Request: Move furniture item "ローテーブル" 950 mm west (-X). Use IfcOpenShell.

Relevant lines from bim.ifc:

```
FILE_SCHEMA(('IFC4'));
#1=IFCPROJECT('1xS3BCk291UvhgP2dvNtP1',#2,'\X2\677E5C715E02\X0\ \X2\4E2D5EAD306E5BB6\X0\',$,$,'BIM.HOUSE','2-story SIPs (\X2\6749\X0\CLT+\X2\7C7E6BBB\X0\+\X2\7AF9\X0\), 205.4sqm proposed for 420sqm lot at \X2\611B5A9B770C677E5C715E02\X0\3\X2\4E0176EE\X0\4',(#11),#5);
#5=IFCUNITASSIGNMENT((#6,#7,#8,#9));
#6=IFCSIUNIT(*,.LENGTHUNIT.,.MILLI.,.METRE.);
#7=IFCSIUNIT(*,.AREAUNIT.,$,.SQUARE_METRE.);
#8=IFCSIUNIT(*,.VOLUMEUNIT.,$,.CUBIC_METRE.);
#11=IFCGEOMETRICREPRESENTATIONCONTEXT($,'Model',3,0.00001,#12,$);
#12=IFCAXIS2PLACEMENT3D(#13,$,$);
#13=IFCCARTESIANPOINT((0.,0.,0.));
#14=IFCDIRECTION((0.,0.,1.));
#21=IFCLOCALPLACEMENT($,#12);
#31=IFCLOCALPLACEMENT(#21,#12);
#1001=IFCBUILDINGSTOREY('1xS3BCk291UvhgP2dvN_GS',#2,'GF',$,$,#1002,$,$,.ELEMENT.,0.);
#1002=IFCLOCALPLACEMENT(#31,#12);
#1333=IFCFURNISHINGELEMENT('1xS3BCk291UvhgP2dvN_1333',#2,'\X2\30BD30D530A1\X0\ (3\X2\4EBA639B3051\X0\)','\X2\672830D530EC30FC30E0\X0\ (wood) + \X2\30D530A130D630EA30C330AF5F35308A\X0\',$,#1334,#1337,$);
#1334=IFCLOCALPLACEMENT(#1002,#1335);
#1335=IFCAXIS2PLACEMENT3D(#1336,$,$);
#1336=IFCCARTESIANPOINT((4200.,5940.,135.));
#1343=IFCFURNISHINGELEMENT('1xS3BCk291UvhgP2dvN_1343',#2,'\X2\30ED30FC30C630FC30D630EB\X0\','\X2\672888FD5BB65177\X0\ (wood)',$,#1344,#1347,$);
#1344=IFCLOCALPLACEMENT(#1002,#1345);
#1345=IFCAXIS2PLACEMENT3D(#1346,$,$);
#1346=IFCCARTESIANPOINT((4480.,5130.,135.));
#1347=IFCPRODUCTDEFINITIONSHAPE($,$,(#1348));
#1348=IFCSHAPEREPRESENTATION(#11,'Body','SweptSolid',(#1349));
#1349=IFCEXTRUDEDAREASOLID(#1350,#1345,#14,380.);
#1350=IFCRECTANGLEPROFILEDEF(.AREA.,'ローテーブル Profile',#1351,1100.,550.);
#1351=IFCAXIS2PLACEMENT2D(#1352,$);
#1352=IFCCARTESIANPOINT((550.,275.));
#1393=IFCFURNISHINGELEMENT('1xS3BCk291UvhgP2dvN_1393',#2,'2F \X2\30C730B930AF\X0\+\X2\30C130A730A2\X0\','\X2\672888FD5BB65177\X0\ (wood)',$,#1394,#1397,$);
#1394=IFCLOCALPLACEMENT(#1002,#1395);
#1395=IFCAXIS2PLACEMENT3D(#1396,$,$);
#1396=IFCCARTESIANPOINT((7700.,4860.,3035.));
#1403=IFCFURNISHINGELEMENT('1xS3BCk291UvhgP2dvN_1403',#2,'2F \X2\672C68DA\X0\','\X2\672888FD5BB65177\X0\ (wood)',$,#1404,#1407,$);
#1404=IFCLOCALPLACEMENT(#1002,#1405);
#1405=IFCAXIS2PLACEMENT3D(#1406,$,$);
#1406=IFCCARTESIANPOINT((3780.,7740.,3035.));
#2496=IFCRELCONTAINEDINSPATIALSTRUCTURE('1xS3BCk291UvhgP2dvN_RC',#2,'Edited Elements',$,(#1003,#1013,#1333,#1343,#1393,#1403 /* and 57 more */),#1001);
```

```python
import ifcopenshell
import ifcopenshell.api.geometry
import ifcopenshell.util.placement
import ifcopenshell.util.unit

model = ifcopenshell.open("bim.ifc")
unit_scale = ifcopenshell.util.unit.calculate_unit_scale(model)

item = model.by_guid("1xS3BCk291UvhgP2dvN_1343")
matrix = ifcopenshell.util.placement.get_local_placement(item.ObjectPlacement)
matrix[0, 3] -= 0.95 / unit_scale
ifcopenshell.api.geometry.edit_object_placement(model, product=item, matrix=matrix, is_si=False)

print(ifcopenshell.util.placement.get_local_placement(item.ObjectPlacement).round(3) + 0.0)

model.write("bim-out.ifc")
```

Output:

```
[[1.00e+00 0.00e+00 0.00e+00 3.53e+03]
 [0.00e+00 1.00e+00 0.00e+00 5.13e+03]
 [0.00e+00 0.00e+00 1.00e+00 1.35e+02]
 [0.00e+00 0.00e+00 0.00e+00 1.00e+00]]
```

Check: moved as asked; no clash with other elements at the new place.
